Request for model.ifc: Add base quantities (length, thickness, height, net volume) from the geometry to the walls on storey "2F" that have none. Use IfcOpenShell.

First a look at what the model holds.

```python
import ifcopenshell
import ifcopenshell.util.element
import ifcopenshell.util.unit

model = ifcopenshell.open("model.ifc")
print(model.schema)
for unit_type in ("LENGTHUNIT", "AREAUNIT", "VOLUMEUNIT"):
    print(unit_type, ifcopenshell.util.unit.calculate_unit_scale(model, unit_type))
storey = next(s for s in model.by_type("IfcBuildingStorey") if s.Name == "2F")
walls = [e for e in ifcopenshell.util.element.get_decomposition(storey) if e.is_a("IfcWall")]
for e in sorted(walls, key=lambda e: e.id()):
    print(e.id(), e.is_a(), e.Name, list(ifcopenshell.util.element.get_psets(e, qtos_only=True)), sep=" | ")
```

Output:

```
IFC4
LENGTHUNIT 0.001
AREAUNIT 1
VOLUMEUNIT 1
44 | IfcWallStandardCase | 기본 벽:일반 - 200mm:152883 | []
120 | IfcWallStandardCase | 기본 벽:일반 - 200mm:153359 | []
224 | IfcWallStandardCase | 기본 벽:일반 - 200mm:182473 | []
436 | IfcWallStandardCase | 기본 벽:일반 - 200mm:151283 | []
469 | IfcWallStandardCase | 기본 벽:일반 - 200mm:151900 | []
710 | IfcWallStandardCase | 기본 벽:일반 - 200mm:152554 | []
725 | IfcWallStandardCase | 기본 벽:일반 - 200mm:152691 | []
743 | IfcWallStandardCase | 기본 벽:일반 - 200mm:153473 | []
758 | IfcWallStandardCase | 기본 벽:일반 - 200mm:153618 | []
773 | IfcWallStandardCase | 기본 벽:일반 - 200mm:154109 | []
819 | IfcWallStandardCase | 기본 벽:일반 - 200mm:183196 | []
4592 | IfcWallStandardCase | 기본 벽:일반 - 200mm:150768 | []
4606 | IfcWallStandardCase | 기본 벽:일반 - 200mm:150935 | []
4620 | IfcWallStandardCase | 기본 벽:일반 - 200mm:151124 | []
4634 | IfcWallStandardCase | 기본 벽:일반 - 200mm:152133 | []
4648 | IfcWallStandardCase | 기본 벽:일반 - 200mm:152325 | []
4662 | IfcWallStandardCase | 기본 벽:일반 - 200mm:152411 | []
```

```python
import ifcopenshell
import ifcopenshell.api.pset
import ifcopenshell.geom
import ifcopenshell.util.element
import ifcopenshell.util.shape
import ifcopenshell.util.unit

model = ifcopenshell.open("model.ifc")
unit_scale = ifcopenshell.util.unit.calculate_unit_scale(model)
volume_scale = ifcopenshell.util.unit.calculate_unit_scale(model, "VOLUMEUNIT")
settings = ifcopenshell.geom.settings()

storey = next(s for s in model.by_type("IfcBuildingStorey") if s.Name == "2F")
walls = [e for e in ifcopenshell.util.element.get_decomposition(storey) if e.is_a("IfcWall")]

for e in sorted(walls, key=lambda e: e.id()):
    if ifcopenshell.util.element.get_psets(e, qtos_only=True, should_inherit=False):
        continue
    # Geometry comes back in metres, in the element's own axes.
    shape = ifcopenshell.geom.create_shape(settings, e)
    values = {
        "Length": ifcopenshell.util.shape.get_x(shape.geometry) / unit_scale,
        "Width": ifcopenshell.util.shape.get_y(shape.geometry) / unit_scale,
        "Height": ifcopenshell.util.shape.get_z(shape.geometry) / unit_scale,
        "NetVolume": ifcopenshell.util.shape.get_volume(shape.geometry) / volume_scale,
    }
    qto = ifcopenshell.api.pset.add_qto(model, product=e, name="Qto_WallBaseQuantities")
    ifcopenshell.api.pset.edit_qto(model, qto=qto, properties=values)
    print(e.id(), {k: round(v, 3) for k, v in values.items()})

model.write("model_edited.ifc")
```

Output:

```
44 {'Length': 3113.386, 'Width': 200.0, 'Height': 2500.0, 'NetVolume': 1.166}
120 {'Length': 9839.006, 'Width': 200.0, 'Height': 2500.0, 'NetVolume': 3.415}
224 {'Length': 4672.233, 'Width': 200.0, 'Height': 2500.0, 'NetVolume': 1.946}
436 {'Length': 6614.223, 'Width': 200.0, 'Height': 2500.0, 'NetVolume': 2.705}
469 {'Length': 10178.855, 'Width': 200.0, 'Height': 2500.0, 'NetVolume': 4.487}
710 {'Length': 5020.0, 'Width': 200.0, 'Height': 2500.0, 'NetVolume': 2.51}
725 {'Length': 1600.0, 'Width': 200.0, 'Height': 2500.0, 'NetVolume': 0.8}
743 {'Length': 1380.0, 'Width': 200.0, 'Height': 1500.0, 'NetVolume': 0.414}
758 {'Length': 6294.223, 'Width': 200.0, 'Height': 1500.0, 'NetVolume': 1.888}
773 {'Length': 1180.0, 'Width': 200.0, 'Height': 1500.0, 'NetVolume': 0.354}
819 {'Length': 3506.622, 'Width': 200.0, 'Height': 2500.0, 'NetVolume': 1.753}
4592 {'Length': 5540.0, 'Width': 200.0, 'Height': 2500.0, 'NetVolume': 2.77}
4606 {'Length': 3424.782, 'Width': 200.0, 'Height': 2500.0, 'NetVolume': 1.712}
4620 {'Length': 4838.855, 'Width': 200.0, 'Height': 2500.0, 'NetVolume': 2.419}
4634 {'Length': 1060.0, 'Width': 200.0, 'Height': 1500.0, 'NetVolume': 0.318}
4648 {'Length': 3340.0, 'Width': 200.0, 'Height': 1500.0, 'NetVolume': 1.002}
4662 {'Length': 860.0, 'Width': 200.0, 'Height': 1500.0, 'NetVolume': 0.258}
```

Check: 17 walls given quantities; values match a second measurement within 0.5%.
